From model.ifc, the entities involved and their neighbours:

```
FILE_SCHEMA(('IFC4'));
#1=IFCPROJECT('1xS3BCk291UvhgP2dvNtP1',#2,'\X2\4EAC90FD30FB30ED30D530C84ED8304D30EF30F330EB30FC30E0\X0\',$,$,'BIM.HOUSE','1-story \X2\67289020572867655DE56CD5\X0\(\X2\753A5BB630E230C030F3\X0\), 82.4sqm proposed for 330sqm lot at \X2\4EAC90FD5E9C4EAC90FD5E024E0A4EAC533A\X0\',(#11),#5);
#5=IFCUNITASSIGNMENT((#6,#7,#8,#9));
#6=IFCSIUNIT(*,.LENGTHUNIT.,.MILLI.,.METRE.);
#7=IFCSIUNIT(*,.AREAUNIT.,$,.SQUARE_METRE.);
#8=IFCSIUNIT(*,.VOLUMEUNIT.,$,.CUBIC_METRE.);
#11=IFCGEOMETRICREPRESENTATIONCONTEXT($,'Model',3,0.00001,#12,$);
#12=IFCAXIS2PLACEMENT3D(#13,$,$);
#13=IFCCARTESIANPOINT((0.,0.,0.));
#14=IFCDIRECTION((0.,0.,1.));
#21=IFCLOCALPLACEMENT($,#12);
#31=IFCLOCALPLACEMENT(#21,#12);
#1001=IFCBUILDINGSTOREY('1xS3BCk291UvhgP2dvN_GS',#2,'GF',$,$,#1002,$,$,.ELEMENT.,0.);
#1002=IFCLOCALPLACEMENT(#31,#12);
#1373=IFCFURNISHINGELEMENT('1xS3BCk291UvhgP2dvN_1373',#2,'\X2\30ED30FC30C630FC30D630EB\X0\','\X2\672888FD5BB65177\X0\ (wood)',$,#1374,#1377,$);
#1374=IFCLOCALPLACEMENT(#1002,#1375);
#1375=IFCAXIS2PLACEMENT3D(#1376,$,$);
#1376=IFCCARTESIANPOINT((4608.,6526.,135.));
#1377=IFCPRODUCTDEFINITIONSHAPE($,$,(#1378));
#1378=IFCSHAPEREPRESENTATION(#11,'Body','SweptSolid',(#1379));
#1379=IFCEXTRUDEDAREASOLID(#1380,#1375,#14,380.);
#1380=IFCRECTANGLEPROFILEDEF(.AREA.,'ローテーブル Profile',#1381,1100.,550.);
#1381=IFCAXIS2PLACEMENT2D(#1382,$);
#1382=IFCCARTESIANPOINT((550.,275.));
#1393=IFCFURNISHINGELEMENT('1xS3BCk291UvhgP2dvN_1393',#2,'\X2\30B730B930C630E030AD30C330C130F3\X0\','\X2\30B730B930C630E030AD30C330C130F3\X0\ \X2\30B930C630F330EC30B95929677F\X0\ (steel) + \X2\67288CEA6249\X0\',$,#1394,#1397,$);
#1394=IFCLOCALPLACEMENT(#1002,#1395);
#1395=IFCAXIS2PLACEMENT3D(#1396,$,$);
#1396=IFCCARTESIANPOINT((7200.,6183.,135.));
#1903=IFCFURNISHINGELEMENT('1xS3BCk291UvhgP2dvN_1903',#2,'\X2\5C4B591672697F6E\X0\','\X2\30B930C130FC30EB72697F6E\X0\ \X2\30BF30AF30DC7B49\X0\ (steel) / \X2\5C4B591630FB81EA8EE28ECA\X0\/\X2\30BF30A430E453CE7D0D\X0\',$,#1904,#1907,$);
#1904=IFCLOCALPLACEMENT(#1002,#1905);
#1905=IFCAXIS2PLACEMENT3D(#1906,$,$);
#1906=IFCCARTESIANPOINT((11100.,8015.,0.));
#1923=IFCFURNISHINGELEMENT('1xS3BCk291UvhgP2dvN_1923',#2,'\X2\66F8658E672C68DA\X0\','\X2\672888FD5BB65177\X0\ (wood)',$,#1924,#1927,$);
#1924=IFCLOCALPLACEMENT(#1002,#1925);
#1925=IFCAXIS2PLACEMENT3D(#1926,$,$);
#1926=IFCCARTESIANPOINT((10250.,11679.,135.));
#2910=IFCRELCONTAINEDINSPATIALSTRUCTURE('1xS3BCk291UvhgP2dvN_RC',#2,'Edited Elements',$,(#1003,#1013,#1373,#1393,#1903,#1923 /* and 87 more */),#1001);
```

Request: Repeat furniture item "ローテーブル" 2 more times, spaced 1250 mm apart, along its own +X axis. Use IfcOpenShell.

```python
import ifcopenshell
import ifcopenshell.api.geometry
import ifcopenshell.api.root
import ifcopenshell.util.element
import ifcopenshell.util.placement
import ifcopenshell.util.unit

model = ifcopenshell.open("model.ifc")
unit_scale = ifcopenshell.util.unit.calculate_unit_scale(model)


def reuse_history(source, copy):
    """copy_class also copies each property set's owner history, people and application; keep the originals."""
    for rel in copy.IsDefinedBy:
        if rel.is_a("IfcRelDefinesByProperties") and (history := rel.RelatingPropertyDefinition.OwnerHistory):
            rel.RelatingPropertyDefinition.OwnerHistory = source.OwnerHistory
            ifcopenshell.util.element.remove_deep2(model, history)


source = model.by_guid("1xS3BCk291UvhgP2dvN_1373")
base = ifcopenshell.util.placement.get_local_placement(source.ObjectPlacement)
step = base[:3, 0] * 1.25 / unit_scale

for i in range(1, 3):
    copy = ifcopenshell.api.root.copy_class(model, product=source)
    copy.Representation = ifcopenshell.util.element.copy_deep(
        model, source.Representation, exclude=["IfcGeometricRepresentationContext", "IfcRepresentationMap"]
    )
    reuse_history(source, copy)
    matrix = base.copy()
    matrix[:3, 3] += i * step
    print("added at", matrix[:3, 3].round(3) + 0.0)
    ifcopenshell.api.geometry.edit_object_placement(model, product=copy, matrix=matrix, is_si=False)

model.write("model_edited.ifc")
```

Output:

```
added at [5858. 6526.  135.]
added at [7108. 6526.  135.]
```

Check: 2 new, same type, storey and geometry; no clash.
